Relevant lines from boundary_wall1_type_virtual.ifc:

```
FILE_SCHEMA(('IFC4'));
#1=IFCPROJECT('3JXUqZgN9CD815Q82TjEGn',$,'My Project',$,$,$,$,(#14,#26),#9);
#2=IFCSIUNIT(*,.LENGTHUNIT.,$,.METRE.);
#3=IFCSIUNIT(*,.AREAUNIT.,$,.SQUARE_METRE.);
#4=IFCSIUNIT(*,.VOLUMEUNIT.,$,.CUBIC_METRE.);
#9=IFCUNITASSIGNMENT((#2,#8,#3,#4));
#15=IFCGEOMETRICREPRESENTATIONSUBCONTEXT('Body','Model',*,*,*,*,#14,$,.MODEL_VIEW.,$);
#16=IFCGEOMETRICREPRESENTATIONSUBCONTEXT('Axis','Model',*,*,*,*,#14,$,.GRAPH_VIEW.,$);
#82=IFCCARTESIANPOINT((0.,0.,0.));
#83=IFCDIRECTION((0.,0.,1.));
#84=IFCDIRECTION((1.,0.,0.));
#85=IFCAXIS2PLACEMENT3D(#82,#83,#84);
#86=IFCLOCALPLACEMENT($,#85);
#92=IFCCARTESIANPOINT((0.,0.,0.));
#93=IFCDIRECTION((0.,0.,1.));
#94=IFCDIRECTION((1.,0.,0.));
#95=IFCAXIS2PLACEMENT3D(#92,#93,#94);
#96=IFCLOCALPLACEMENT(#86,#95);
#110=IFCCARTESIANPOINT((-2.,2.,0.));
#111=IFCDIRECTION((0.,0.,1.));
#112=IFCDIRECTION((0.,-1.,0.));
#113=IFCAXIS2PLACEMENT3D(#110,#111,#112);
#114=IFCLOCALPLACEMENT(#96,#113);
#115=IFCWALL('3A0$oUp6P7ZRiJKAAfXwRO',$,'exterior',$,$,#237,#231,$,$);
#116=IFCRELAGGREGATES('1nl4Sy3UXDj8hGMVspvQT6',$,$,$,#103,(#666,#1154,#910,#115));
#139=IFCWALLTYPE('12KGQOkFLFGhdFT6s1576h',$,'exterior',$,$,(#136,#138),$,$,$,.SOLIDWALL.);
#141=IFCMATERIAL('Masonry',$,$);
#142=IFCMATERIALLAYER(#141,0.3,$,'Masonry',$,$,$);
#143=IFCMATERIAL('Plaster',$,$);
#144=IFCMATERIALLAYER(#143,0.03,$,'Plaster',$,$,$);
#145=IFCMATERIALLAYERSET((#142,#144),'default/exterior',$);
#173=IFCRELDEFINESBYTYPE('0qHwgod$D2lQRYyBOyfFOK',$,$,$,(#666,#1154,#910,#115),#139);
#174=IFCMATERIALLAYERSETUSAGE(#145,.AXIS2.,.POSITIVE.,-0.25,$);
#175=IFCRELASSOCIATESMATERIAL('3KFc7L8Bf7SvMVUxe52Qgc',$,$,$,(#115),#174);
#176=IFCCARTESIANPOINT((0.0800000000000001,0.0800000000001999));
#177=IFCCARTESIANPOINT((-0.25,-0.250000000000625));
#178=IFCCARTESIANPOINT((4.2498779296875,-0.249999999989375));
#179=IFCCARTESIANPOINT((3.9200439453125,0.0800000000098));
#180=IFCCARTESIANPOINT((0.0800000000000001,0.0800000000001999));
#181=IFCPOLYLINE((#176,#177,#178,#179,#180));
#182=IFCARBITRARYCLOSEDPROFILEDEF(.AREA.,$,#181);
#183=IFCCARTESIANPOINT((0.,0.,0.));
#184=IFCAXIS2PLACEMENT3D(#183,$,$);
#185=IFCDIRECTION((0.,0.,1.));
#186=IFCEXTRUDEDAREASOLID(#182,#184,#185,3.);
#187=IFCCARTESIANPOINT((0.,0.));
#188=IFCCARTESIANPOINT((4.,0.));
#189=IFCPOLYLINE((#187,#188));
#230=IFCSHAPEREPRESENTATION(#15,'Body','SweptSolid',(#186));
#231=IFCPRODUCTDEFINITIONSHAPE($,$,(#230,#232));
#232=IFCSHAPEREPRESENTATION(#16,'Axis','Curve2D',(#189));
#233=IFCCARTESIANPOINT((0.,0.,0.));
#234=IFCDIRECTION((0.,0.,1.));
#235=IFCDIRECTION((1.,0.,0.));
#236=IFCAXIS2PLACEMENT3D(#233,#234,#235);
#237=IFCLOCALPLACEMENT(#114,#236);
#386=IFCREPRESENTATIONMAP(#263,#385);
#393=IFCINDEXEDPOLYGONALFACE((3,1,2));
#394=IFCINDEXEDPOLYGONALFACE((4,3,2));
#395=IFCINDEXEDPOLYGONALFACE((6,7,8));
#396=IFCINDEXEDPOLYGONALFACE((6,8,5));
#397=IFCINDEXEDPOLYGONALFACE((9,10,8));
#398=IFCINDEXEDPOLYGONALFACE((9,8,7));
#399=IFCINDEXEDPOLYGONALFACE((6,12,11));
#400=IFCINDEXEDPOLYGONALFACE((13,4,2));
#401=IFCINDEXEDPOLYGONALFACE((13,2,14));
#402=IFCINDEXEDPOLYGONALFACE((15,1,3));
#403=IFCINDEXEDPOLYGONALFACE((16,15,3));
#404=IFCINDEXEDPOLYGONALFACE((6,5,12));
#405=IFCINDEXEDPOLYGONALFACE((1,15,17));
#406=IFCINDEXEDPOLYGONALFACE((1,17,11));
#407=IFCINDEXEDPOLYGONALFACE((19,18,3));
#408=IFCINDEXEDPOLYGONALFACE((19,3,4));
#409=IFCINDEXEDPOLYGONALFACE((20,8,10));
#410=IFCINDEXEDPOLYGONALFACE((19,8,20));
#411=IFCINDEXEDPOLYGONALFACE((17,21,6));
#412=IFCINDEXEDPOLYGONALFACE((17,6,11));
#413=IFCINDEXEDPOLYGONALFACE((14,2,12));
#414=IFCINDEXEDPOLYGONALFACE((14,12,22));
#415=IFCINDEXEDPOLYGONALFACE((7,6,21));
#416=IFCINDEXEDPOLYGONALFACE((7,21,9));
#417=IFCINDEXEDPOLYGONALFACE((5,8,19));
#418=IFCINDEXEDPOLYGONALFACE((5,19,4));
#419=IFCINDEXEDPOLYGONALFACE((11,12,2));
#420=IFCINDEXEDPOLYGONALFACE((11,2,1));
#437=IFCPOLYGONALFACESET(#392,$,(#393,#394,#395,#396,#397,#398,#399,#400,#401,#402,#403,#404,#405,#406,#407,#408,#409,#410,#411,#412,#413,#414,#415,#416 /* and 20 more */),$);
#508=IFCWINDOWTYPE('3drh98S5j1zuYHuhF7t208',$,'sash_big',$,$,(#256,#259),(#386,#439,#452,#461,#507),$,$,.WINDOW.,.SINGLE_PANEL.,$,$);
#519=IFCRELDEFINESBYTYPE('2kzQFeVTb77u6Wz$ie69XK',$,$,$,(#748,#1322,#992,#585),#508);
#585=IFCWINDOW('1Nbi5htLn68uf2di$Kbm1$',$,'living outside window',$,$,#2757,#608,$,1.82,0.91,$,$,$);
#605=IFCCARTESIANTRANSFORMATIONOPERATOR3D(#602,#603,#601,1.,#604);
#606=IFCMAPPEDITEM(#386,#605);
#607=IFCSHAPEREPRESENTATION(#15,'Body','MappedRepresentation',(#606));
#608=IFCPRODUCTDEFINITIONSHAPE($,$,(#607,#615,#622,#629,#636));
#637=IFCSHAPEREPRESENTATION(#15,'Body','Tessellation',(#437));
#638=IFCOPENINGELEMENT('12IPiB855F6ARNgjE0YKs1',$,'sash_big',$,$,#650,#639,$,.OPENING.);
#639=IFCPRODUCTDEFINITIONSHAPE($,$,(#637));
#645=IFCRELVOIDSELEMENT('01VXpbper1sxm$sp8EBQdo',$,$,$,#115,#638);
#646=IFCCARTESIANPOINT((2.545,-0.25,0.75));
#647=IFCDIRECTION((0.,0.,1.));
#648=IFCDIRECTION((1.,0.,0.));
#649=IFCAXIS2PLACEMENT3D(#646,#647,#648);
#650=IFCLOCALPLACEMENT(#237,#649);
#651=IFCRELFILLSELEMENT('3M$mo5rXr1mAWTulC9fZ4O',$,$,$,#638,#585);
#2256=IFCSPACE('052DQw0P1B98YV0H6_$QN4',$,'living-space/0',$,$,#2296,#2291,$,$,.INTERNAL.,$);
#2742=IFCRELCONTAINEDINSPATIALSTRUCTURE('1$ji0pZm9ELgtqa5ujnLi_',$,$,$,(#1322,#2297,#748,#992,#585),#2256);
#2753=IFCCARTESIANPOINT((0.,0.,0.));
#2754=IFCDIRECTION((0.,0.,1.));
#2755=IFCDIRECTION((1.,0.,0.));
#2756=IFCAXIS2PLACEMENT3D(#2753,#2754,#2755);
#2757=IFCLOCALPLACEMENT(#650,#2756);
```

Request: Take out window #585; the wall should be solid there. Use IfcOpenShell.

```python
import ifcopenshell
import ifcopenshell.api.feature
import ifcopenshell.api.root
import ifcopenshell.geom
import ifcopenshell.util.shape

model = ifcopenshell.open("boundary_wall1_type_virtual.ifc")
settings = ifcopenshell.geom.settings()


def volume(element):
    """Net volume in cubic metres, openings subtracted."""
    shape = ifcopenshell.geom.create_shape(settings, element)
    return ifcopenshell.util.shape.get_volume(shape.geometry)


window = model.by_id(585)
opening = window.FillsVoids[0].RelatingOpeningElement
wall = opening.VoidsElements[0].RelatingBuildingElement
before = volume(wall)

ifcopenshell.api.root.remove_product(model, product=window)
ifcopenshell.api.feature.remove_feature(model, feature=opening)

after = volume(wall)

print(f"wall volume {before:.3f} -> {after:.3f} m3")

model.write("boundary_wall1_type_virtual_rev.ifc")
```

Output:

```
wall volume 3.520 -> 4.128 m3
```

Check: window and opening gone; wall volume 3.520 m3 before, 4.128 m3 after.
